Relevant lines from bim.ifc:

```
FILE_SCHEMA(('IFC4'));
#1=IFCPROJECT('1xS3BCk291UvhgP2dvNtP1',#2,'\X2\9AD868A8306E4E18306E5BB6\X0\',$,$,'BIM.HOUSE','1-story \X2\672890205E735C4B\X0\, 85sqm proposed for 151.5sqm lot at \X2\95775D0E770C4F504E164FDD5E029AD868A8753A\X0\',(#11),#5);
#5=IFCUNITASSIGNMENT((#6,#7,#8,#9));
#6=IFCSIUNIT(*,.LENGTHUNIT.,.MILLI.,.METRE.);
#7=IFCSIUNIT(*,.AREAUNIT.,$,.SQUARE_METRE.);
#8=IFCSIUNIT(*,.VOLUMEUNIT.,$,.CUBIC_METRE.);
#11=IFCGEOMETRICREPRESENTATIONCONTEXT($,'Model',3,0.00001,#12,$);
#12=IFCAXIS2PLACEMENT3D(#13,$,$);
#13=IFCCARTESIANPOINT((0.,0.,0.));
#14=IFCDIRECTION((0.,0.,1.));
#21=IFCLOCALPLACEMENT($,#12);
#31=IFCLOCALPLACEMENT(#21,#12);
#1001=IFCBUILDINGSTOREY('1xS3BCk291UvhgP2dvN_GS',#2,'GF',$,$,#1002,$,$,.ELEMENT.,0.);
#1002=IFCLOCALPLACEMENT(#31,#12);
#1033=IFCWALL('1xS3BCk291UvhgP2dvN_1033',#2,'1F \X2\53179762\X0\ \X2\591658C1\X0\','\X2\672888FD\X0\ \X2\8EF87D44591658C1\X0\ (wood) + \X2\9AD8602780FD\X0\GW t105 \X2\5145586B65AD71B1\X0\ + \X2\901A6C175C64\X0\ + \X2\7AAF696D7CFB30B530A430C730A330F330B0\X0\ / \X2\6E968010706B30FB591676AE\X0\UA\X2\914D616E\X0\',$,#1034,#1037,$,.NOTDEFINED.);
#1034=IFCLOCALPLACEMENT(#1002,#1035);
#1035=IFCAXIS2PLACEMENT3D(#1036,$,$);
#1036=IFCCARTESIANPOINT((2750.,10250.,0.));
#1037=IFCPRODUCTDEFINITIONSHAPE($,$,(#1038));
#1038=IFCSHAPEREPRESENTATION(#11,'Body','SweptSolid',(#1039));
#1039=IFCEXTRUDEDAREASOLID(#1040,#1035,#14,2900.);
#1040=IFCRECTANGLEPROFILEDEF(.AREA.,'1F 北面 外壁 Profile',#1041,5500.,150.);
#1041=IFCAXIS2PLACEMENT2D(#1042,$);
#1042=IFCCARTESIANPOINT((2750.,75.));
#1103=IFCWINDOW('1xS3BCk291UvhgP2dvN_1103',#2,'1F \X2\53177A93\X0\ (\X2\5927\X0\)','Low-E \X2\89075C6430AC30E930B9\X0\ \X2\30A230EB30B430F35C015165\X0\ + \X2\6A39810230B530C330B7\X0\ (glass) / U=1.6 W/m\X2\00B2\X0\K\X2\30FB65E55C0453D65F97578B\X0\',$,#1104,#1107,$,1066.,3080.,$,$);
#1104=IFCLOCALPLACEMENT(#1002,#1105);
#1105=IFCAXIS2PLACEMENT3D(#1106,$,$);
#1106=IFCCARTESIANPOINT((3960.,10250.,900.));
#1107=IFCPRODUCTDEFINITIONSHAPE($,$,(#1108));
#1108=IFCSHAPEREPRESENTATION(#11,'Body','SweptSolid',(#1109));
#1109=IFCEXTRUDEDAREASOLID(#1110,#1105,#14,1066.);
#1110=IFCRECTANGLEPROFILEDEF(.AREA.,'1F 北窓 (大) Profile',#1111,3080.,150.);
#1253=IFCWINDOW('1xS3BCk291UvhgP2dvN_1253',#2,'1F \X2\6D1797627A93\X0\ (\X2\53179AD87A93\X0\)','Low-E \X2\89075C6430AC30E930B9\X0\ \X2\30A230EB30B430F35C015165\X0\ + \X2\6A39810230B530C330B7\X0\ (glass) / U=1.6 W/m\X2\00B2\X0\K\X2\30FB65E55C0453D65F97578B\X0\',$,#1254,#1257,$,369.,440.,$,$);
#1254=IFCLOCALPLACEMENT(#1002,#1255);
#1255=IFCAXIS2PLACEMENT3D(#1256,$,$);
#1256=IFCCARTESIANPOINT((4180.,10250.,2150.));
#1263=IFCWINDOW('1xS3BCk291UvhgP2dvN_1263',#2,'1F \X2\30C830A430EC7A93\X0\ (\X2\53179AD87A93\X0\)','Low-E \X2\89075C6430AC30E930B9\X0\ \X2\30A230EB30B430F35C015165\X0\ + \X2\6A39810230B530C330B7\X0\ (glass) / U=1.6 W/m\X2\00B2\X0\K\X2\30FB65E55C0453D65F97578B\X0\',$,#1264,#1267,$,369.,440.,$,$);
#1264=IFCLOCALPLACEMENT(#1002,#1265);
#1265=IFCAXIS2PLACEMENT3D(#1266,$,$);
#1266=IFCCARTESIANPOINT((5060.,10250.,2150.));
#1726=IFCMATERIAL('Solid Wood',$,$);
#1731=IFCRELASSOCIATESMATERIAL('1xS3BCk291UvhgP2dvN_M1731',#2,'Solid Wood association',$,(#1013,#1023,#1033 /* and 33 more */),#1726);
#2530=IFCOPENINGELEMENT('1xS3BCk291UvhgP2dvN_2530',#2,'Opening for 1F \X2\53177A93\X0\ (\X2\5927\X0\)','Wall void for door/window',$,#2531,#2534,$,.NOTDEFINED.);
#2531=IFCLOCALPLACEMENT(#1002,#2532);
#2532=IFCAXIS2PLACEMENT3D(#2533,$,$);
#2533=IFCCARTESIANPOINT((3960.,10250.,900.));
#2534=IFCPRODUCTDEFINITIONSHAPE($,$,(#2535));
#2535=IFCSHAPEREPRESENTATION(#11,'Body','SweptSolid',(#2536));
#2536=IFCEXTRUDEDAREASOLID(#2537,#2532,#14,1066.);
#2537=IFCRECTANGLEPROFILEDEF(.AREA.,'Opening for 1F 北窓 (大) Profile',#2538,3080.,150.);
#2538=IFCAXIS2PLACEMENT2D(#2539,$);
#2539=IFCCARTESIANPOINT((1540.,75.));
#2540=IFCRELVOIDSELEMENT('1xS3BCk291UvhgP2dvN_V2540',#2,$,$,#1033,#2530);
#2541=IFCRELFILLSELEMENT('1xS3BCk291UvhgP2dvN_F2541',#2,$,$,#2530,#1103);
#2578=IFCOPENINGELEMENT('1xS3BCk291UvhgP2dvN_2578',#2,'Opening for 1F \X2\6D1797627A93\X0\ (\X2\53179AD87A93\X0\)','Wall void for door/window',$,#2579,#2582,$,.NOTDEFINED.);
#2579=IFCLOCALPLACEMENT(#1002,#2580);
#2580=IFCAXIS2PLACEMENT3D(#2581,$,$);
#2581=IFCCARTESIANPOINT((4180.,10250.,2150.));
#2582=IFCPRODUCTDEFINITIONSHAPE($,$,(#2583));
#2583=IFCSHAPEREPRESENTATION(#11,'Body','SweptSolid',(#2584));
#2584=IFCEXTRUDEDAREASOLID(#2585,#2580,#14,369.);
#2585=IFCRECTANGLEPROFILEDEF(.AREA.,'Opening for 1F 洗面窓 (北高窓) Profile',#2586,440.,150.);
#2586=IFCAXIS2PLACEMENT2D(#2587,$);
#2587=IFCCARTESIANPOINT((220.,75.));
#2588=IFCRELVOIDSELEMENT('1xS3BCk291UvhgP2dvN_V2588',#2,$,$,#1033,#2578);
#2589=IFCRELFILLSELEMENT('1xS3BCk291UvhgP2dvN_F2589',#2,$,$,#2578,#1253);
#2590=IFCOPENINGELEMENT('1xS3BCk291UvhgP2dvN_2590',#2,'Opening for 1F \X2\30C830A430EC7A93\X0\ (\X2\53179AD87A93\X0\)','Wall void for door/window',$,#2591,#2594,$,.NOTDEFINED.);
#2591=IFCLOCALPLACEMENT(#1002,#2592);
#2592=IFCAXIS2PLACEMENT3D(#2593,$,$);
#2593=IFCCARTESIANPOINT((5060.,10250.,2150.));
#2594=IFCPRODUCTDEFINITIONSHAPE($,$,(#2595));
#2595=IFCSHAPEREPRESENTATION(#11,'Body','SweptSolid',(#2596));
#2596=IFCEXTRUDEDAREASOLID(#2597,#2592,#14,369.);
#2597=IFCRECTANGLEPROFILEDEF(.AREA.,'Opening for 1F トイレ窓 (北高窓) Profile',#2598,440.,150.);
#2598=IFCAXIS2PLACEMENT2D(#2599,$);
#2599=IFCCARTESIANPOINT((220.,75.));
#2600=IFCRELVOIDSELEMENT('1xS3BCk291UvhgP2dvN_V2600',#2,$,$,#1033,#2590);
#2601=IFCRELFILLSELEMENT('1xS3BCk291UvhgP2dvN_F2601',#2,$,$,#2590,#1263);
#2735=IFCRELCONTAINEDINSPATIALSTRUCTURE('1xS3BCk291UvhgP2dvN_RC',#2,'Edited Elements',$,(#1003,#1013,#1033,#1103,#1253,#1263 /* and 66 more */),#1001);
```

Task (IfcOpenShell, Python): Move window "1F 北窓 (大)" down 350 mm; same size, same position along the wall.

```python
import numpy as np
import ifcopenshell
import ifcopenshell.api.geometry
import ifcopenshell.util.placement
import ifcopenshell.util.unit

model = ifcopenshell.open("bim.ifc")
unit_scale = ifcopenshell.util.unit.calculate_unit_scale(model)

window = model.by_guid("1xS3BCk291UvhgP2dvN_1103")
opening = window.FillsVoids[0].RelatingOpeningElement
dz = -0.35 / unit_scale

shift = np.array([0.0, 0.0, dz])
# The window is not placed relative to its opening, so move both.
for product in (opening, window):
    matrix = ifcopenshell.util.placement.get_local_placement(product.ObjectPlacement)
    matrix[:3, 3] += shift
    ifcopenshell.api.geometry.edit_object_placement(model, product=product, matrix=matrix, is_si=False)

print(f"moved by {dz * unit_scale:+.3f} m")

model.write("bim_rev.ifc")
```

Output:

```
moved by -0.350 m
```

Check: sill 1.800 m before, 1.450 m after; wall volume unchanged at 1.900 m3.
